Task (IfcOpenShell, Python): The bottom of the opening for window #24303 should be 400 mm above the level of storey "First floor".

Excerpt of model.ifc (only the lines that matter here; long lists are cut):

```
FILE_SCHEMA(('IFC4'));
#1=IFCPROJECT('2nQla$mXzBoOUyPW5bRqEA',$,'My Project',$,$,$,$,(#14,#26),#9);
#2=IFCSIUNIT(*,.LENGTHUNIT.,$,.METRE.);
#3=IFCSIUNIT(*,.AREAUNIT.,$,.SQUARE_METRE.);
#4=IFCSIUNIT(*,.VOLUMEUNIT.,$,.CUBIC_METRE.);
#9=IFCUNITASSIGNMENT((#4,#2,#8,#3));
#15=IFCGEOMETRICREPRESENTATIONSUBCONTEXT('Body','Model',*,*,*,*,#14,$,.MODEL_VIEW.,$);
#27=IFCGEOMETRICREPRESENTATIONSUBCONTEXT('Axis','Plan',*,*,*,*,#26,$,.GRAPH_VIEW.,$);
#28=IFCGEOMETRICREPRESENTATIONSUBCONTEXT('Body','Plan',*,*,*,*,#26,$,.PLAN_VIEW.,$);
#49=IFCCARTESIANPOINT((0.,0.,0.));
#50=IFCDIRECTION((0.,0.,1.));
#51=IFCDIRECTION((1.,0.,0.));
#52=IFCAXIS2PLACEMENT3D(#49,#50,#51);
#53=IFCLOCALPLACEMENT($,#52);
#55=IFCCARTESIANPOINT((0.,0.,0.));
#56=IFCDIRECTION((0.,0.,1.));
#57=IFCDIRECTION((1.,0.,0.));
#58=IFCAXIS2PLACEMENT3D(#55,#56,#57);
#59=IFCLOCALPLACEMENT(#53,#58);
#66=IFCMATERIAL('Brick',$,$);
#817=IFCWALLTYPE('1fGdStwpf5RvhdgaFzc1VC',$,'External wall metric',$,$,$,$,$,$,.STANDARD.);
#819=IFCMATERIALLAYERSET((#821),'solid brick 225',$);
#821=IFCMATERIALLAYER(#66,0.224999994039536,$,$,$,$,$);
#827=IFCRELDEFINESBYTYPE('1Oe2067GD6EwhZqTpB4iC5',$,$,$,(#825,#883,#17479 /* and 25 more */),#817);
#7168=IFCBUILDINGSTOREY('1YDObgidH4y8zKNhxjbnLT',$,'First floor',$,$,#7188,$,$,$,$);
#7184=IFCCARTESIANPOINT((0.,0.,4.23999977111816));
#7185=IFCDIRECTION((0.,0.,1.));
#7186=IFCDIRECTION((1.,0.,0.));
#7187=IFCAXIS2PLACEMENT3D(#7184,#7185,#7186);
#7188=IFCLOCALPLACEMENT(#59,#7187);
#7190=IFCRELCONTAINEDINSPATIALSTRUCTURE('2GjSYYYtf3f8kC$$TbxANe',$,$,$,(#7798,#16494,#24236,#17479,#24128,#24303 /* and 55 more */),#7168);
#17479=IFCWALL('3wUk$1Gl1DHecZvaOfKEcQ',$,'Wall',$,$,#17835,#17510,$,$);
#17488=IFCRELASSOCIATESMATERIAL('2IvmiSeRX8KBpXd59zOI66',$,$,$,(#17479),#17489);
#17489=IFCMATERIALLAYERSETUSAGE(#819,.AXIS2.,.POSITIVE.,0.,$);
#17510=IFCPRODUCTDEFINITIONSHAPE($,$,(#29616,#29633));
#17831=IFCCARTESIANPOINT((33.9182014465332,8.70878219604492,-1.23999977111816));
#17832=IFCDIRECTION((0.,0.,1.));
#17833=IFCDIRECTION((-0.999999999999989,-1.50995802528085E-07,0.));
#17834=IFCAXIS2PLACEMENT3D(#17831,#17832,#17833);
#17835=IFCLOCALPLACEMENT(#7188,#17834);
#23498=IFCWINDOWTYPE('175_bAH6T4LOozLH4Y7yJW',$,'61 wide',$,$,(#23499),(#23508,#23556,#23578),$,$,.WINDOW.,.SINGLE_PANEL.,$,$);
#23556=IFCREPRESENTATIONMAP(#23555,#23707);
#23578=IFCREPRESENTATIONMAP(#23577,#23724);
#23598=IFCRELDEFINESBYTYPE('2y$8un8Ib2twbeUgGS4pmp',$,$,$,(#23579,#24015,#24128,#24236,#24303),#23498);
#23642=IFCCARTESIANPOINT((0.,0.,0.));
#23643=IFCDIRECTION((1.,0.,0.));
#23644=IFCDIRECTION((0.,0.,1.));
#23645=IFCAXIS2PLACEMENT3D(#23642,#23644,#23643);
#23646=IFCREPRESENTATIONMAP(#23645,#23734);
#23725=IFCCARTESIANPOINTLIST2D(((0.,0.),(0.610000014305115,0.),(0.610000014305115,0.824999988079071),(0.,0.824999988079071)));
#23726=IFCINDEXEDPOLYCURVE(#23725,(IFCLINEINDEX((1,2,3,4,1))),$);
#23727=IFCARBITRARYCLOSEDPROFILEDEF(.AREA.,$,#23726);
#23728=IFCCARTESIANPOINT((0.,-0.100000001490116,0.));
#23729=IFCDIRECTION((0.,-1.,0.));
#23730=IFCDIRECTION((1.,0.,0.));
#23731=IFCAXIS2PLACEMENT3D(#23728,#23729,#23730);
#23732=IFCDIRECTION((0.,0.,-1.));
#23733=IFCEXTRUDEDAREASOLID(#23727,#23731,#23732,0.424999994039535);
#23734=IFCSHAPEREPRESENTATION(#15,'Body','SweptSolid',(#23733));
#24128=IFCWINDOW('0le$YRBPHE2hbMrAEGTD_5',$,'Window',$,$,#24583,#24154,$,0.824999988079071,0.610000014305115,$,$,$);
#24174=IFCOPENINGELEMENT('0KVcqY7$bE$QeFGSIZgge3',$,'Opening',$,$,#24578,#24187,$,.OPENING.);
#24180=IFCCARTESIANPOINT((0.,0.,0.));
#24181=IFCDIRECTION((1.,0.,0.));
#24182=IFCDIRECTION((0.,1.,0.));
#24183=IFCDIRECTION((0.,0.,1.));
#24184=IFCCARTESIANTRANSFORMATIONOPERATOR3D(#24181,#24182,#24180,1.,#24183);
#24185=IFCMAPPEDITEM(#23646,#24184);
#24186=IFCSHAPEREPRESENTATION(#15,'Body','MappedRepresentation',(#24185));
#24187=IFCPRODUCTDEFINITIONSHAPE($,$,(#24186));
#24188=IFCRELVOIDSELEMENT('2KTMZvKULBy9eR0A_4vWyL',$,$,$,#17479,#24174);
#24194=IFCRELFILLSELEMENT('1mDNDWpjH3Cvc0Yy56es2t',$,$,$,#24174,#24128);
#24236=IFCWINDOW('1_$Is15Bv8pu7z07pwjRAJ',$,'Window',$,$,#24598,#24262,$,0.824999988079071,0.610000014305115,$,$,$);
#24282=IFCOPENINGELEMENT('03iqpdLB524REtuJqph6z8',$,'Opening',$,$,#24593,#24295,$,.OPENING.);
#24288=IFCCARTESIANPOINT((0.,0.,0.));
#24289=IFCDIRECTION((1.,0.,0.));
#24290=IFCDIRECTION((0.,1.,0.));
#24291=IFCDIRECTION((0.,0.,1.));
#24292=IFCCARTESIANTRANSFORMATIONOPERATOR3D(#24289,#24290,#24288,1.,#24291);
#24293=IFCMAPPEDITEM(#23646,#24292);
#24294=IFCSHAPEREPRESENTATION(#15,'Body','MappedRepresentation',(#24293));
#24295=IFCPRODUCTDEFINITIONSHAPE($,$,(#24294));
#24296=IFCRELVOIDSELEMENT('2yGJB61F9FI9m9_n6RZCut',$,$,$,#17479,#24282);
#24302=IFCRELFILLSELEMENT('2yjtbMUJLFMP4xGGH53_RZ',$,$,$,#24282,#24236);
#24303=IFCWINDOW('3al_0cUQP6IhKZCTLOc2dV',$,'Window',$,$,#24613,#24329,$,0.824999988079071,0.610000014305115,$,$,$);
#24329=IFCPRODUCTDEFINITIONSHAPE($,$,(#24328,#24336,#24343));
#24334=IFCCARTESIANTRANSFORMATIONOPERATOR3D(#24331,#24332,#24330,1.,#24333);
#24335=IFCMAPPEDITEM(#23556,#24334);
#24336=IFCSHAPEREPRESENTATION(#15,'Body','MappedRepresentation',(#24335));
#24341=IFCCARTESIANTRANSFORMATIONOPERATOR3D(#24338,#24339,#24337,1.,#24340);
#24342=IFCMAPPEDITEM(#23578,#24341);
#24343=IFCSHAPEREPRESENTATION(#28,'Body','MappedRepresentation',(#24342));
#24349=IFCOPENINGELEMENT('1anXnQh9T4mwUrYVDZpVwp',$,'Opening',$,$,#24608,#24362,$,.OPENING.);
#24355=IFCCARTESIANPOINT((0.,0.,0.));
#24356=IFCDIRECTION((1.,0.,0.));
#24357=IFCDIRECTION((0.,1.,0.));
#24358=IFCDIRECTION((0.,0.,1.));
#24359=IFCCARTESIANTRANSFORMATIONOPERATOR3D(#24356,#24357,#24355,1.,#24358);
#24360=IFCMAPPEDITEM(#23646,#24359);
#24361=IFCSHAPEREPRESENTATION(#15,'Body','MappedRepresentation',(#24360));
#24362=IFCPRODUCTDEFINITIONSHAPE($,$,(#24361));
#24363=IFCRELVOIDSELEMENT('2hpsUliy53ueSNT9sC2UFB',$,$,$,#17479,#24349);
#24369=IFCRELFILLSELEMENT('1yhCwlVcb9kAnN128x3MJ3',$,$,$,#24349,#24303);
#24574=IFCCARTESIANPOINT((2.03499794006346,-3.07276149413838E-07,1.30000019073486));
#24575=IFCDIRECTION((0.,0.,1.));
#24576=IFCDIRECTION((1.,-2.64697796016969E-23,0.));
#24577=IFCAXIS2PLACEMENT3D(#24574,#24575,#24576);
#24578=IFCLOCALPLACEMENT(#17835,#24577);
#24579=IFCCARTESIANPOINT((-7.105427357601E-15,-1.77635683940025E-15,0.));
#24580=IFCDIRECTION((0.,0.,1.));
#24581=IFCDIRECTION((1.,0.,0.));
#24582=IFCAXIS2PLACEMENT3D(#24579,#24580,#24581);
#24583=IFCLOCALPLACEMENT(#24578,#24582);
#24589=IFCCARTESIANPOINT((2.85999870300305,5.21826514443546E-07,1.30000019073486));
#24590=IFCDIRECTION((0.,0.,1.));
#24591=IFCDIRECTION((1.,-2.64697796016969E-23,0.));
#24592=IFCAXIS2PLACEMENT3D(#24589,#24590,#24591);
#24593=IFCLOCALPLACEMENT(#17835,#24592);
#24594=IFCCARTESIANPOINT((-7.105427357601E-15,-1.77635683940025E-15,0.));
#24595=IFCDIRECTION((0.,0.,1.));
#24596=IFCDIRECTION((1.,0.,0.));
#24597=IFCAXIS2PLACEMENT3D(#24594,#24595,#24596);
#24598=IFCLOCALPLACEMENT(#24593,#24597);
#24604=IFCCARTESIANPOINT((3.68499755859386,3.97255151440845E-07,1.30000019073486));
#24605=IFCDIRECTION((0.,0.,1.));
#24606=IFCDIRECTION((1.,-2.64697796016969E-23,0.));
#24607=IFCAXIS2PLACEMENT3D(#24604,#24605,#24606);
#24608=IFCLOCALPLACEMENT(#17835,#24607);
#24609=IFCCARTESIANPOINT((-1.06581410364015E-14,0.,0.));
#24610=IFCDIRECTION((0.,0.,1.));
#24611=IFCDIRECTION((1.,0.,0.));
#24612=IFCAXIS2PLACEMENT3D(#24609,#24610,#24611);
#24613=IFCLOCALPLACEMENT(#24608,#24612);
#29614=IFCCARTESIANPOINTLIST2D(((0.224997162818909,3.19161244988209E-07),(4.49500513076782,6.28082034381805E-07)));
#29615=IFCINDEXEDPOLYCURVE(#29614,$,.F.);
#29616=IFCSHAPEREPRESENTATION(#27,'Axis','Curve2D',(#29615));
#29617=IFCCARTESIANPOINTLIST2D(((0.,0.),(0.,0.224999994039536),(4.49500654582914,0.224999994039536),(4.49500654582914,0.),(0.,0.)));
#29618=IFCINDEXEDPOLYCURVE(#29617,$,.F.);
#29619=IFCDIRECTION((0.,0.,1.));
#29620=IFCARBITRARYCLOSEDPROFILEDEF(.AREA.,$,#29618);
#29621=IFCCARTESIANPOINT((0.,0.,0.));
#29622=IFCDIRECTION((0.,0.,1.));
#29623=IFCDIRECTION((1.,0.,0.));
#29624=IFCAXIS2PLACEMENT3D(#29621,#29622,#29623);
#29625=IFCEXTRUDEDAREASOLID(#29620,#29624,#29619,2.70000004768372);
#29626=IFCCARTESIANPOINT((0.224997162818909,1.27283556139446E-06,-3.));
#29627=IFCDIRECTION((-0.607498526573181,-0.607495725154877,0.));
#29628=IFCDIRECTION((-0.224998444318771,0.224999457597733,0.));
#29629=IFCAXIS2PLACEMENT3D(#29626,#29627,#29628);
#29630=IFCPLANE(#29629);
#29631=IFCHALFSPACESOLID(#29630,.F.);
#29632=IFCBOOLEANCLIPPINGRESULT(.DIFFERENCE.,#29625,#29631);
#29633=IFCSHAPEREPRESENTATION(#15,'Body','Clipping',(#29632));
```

```python
import numpy as np
import ifcopenshell
import ifcopenshell.api.geometry
import ifcopenshell.geom
import ifcopenshell.util.element
import ifcopenshell.util.placement
import ifcopenshell.util.shape
import ifcopenshell.util.unit

model = ifcopenshell.open("model.ifc")
unit_scale = ifcopenshell.util.unit.calculate_unit_scale(model)

window = model.by_guid("3al_0cUQP6IhKZCTLOc2dV")
opening = window.FillsVoids[0].RelatingOpeningElement
storey = ifcopenshell.util.element.get_container(window, ifc_class="IfcBuildingStorey")
level = ifcopenshell.util.placement.get_local_placement(storey.ObjectPlacement)[2, 3]

# The opening's origin need not be at the sill, so measure its lowest point.
shape = ifcopenshell.geom.create_shape(ifcopenshell.geom.settings(), opening)
bottom = ifcopenshell.util.shape.get_shape_bottom_elevation(shape, shape.geometry) / unit_scale
dz = level + 0.4 / unit_scale - bottom

shift = np.array([0.0, 0.0, dz])
# The window is placed relative to its opening, so it follows when the opening moves.
matrix = ifcopenshell.util.placement.get_local_placement(opening.ObjectPlacement)
matrix[:3, 3] += shift
ifcopenshell.api.geometry.edit_object_placement(
    model, product=opening, matrix=matrix, is_si=False, should_transform_children=True
)

print(f"moved by {dz * unit_scale:+.3f} m")

model.write("model-out.ifc")
```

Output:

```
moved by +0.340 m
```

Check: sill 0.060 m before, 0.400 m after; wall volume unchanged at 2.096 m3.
